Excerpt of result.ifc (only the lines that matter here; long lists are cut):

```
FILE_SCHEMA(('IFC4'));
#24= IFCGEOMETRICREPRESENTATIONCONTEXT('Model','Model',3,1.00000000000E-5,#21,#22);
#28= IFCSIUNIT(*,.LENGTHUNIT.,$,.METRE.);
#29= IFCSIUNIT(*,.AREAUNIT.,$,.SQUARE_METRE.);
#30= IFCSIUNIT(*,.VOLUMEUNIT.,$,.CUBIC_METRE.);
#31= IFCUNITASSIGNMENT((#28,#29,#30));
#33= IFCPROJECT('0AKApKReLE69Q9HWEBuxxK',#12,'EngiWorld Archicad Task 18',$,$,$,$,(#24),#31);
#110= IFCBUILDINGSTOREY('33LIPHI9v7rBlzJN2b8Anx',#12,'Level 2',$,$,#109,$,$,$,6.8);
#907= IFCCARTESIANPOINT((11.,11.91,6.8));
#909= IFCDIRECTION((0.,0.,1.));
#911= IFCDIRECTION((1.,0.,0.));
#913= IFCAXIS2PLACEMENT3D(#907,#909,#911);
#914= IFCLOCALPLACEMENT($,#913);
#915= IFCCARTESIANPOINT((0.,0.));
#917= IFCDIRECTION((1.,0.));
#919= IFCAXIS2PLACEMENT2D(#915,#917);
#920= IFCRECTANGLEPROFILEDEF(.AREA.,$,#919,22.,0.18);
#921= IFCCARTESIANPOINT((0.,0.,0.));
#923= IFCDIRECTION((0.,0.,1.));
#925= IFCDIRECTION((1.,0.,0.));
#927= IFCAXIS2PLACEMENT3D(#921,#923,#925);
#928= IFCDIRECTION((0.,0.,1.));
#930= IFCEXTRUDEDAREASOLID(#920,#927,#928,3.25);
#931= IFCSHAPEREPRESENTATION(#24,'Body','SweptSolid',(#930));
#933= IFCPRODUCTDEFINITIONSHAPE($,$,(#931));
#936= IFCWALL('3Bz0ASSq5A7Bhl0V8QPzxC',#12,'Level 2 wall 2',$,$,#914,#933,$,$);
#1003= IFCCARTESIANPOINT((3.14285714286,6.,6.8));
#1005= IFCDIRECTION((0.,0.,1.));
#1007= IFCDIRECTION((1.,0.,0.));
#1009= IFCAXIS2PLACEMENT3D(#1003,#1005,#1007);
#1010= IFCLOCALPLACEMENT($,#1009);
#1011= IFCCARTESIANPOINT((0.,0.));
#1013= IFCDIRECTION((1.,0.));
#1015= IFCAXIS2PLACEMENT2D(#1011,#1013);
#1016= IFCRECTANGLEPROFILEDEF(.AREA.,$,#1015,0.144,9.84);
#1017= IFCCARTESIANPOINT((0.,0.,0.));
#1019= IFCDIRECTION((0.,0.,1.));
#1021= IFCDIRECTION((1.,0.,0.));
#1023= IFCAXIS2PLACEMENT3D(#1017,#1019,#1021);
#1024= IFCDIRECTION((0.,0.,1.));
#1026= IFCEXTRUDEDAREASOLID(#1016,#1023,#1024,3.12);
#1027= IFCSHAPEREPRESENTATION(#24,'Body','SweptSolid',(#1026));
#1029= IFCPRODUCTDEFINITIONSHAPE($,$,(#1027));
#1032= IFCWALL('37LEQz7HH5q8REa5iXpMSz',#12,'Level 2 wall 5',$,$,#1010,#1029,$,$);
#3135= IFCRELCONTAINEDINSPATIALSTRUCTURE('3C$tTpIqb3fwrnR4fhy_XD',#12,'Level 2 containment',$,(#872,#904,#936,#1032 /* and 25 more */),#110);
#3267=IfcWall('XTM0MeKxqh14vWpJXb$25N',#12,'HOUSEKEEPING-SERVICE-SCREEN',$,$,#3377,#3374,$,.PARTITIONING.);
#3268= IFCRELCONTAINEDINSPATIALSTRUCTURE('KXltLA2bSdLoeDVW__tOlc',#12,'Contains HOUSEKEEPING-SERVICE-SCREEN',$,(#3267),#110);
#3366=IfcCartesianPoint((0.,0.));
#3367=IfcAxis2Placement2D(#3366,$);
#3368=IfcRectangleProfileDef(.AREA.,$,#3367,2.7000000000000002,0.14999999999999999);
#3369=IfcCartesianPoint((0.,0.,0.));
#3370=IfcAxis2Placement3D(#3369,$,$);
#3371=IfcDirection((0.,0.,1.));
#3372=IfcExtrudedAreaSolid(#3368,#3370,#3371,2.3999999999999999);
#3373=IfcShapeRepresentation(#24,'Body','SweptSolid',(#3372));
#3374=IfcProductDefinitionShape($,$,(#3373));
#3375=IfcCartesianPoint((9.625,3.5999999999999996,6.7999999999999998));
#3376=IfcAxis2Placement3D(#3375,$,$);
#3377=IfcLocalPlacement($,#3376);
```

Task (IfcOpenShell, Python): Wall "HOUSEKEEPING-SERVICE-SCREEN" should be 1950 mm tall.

```python
import ifcopenshell
import ifcopenshell.geom
import ifcopenshell.util.shape

model = ifcopenshell.open("result.ifc")
settings = ifcopenshell.geom.settings()


def volume(element):
    """Net volume in cubic metres, openings subtracted."""
    shape = ifcopenshell.geom.create_shape(settings, element)
    return ifcopenshell.util.shape.get_volume(shape.geometry)


wall = model.by_id(3267)
before = volume(wall)

body = next(r for r in wall.Representation.Representations if r.RepresentationIdentifier == "Body")
solid = body.Items[0]
old_height = solid.Depth
solid.Depth = 1.95
after = volume(wall)

print(f"height {old_height:g} -> {solid.Depth:g}, volume {before:.3f} -> {after:.3f} m3")

model.write("result_edited.ifc")
```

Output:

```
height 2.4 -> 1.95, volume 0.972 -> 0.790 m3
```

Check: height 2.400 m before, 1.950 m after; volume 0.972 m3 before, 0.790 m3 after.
